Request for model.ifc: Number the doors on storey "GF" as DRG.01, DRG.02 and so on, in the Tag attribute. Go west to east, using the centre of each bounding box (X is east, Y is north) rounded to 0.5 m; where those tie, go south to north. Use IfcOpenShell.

First a look at what the model holds.

```python
import ifcopenshell
import ifcopenshell.util.element
import ifcopenshell.util.placement

model = ifcopenshell.open("model.ifc")
print(model.schema)
storey = next(s for s in model.by_type("IfcBuildingStorey") if s.Name == "GF")
doors = [e for e in ifcopenshell.util.element.get_decomposition(storey) if e.is_a("IfcDoor")]
for e in sorted(doors, key=lambda e: e.id()):
    origin = ifcopenshell.util.placement.get_local_placement(e.ObjectPlacement)[:3, 3]
    print(e.id(), e.Tag, e.Name, origin.round(2) + 0.0, sep=" | ")
```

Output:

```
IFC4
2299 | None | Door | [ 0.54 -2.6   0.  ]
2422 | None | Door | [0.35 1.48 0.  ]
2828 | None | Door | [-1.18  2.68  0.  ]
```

```python
import ifcopenshell
import ifcopenshell.geom
import ifcopenshell.util.element
import ifcopenshell.util.shape

model = ifcopenshell.open("model.ifc")
settings = ifcopenshell.geom.settings()
settings.set("use-world-coords", True)


def centre(element):
    shape = ifcopenshell.geom.create_shape(settings, element)
    return ifcopenshell.util.shape.get_bbox_centroid(shape.geometry)


storey = next(s for s in model.by_type("IfcBuildingStorey") if s.Name == "GF")
doors = [e for e in ifcopenshell.util.element.get_decomposition(storey) if e.is_a("IfcDoor")]

# Insertion points can sit at a corner or the storey origin, so sort by the geometry (in metres).
centres = {e: centre(e) for e in doors}
doors.sort(key=lambda e: (round(centres[e][0] / 0.5), centres[e][1]))

for i, e in enumerate(doors, start=1):
    number = f"DRG.{i:02d}"
    e.Tag = number
    print(e.id(), number)

model.write("model_updated.ifc")
```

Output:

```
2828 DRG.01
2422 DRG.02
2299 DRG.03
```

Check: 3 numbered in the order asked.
